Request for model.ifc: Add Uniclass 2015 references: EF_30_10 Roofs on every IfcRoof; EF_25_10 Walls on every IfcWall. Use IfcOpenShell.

First a look at what the model holds.

```python
import ifcopenshell

model = ifcopenshell.open("model.ifc")
print(model.schema)
print("classifications:", [c.Name for c in model.by_type("IfcClassification")])
for ifc_class in ("IfcDoor", "IfcRoof", "IfcStair", "IfcWall", "IfcWindow"):
    print(ifc_class, len(model.by_type(ifc_class)))
```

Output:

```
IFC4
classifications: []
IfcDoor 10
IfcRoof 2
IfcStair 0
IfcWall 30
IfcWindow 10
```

```python
import ifcopenshell
import ifcopenshell.api.classification

model = ifcopenshell.open("model.ifc")

system = ifcopenshell.api.classification.add_classification(model, classification="Uniclass 2015")

codes = {
    "IfcRoof": ("EF_30_10", "Roofs"),
    "IfcWall": ("EF_25_10", "Walls"),
}
for ifc_class, (code, name) in codes.items():
    products = model.by_type(ifc_class)
    ifcopenshell.api.classification.add_reference(
        model, products=products, classification=system, identification=code, name=name
    )
    print(code, len(products))

model.write("model_v2.ifc")
```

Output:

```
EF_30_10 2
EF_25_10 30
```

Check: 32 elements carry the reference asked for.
